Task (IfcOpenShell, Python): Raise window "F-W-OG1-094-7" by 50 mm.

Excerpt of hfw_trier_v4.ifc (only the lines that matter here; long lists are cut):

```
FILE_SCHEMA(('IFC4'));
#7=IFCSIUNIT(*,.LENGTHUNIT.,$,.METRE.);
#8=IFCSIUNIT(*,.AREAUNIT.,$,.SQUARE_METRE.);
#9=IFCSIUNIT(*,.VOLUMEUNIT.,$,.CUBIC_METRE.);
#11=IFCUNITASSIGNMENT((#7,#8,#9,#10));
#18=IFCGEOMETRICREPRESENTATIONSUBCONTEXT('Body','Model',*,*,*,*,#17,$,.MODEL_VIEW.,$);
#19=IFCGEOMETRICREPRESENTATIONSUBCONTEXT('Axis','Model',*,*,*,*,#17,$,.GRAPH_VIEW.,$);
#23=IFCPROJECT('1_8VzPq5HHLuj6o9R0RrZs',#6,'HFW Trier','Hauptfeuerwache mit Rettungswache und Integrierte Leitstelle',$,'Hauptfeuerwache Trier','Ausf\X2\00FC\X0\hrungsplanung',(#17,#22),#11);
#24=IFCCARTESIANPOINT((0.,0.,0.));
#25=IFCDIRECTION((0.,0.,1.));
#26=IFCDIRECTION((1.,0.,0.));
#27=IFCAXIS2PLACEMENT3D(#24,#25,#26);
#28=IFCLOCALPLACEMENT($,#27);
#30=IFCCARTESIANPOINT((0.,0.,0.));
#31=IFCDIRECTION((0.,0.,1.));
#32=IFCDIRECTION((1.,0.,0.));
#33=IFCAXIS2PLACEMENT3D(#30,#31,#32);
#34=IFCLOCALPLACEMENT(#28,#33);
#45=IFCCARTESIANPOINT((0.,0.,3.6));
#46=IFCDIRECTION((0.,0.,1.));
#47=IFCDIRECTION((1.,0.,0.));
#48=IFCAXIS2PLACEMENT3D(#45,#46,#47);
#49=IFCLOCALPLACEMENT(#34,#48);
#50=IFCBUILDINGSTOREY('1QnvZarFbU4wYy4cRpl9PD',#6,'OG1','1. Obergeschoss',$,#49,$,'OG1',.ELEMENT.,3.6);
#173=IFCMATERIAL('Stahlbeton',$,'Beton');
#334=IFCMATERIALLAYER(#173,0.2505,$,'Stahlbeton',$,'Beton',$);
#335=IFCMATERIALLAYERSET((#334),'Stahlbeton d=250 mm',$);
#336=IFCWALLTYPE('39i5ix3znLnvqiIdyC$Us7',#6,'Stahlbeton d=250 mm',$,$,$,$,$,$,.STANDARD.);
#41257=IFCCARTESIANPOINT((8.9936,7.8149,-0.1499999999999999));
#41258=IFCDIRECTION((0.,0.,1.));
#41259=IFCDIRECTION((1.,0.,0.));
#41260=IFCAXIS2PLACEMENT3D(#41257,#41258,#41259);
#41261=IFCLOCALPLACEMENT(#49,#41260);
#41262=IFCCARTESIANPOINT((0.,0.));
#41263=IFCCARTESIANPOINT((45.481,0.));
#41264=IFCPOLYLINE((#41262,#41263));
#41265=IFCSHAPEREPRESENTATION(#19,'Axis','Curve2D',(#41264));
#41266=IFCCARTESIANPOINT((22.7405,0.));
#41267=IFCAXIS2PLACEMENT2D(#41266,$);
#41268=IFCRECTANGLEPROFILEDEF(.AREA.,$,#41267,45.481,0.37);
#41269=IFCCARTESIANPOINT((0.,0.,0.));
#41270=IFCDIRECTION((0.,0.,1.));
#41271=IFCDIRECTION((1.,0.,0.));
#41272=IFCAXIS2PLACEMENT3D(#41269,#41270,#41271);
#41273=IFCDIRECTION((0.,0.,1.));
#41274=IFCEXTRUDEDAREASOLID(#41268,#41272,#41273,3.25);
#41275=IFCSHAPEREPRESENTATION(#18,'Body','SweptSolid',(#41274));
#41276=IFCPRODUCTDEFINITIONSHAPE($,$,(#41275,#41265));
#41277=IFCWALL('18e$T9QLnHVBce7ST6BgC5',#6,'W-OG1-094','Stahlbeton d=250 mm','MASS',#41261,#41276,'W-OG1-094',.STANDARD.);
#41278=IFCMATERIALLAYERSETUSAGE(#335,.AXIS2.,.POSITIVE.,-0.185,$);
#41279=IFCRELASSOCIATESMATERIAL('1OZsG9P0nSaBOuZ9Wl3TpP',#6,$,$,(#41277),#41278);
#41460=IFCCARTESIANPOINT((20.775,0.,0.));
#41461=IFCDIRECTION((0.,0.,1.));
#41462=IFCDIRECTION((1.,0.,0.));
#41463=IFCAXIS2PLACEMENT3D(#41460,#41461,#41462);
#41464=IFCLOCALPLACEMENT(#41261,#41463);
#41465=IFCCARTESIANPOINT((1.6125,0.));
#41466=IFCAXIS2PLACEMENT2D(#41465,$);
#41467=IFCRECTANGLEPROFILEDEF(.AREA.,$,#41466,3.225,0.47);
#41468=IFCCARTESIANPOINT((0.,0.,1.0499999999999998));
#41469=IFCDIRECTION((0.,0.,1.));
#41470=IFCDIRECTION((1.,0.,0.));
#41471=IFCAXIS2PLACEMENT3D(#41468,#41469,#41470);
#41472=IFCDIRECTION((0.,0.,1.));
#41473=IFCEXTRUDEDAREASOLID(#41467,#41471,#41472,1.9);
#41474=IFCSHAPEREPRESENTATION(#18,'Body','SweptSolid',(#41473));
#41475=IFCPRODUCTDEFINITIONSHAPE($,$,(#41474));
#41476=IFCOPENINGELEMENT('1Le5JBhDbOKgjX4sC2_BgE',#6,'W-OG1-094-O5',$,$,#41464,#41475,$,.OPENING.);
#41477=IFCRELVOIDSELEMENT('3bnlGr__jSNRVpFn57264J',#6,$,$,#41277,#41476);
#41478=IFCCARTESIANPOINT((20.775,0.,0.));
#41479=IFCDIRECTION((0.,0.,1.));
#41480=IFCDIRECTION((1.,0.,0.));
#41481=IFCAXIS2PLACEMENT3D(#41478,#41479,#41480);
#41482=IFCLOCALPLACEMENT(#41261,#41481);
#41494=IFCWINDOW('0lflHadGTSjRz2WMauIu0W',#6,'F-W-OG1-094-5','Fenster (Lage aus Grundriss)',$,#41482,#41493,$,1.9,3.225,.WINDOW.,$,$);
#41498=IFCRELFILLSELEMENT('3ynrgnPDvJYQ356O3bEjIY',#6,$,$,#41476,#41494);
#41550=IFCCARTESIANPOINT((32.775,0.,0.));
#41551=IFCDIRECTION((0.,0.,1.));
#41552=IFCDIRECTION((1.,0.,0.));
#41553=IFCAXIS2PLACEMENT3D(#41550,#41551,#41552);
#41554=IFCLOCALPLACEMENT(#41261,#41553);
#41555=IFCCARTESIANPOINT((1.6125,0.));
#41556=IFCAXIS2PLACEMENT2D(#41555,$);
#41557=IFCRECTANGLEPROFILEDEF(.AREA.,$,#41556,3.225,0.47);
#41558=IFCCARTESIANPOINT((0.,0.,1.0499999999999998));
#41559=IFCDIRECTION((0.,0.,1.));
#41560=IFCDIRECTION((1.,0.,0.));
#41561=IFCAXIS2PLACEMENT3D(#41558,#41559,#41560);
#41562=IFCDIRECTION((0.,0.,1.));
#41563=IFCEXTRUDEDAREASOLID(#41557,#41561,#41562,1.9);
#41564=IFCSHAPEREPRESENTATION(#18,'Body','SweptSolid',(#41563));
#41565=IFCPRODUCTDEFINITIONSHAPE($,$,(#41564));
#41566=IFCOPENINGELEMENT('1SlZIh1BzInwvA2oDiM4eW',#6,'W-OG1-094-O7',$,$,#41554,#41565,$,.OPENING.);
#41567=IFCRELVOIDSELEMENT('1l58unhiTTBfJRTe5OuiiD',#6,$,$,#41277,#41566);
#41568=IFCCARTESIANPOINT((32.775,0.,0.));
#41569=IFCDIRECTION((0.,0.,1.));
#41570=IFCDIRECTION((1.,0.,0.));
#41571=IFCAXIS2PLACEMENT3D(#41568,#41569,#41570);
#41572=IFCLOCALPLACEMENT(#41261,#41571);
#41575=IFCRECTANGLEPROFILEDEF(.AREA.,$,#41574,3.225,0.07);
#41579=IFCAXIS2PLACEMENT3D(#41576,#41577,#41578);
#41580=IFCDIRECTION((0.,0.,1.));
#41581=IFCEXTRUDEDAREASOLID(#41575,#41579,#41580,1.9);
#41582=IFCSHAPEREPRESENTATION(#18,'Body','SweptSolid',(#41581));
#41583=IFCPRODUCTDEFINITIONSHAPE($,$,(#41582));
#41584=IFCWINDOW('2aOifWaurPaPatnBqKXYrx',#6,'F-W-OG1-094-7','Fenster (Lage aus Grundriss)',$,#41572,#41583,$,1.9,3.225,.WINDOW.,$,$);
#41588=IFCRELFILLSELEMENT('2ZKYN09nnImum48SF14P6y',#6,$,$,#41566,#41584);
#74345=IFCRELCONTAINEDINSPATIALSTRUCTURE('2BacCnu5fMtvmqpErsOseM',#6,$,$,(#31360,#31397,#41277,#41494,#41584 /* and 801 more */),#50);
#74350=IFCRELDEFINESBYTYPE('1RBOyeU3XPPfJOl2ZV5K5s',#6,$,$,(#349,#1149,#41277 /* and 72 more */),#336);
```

```python
import numpy as np
import ifcopenshell
import ifcopenshell.api.geometry
import ifcopenshell.util.placement
import ifcopenshell.util.unit

model = ifcopenshell.open("hfw_trier_v4.ifc")
unit_scale = ifcopenshell.util.unit.calculate_unit_scale(model)

window = model.by_guid("2aOifWaurPaPatnBqKXYrx")
opening = window.FillsVoids[0].RelatingOpeningElement
dz = 0.05 / unit_scale

shift = np.array([0.0, 0.0, dz])
# The window is not placed relative to its opening, so move both.
for product in (opening, window):
    matrix = ifcopenshell.util.placement.get_local_placement(product.ObjectPlacement)
    matrix[:3, 3] += shift
    ifcopenshell.api.geometry.edit_object_placement(model, product=product, matrix=matrix, is_si=False)

print(f"moved by {dz * unit_scale:+.3f} m")

model.write("hfw_trier_v4_v2.ifc")
```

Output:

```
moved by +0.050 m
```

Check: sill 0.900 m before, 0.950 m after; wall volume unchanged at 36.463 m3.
